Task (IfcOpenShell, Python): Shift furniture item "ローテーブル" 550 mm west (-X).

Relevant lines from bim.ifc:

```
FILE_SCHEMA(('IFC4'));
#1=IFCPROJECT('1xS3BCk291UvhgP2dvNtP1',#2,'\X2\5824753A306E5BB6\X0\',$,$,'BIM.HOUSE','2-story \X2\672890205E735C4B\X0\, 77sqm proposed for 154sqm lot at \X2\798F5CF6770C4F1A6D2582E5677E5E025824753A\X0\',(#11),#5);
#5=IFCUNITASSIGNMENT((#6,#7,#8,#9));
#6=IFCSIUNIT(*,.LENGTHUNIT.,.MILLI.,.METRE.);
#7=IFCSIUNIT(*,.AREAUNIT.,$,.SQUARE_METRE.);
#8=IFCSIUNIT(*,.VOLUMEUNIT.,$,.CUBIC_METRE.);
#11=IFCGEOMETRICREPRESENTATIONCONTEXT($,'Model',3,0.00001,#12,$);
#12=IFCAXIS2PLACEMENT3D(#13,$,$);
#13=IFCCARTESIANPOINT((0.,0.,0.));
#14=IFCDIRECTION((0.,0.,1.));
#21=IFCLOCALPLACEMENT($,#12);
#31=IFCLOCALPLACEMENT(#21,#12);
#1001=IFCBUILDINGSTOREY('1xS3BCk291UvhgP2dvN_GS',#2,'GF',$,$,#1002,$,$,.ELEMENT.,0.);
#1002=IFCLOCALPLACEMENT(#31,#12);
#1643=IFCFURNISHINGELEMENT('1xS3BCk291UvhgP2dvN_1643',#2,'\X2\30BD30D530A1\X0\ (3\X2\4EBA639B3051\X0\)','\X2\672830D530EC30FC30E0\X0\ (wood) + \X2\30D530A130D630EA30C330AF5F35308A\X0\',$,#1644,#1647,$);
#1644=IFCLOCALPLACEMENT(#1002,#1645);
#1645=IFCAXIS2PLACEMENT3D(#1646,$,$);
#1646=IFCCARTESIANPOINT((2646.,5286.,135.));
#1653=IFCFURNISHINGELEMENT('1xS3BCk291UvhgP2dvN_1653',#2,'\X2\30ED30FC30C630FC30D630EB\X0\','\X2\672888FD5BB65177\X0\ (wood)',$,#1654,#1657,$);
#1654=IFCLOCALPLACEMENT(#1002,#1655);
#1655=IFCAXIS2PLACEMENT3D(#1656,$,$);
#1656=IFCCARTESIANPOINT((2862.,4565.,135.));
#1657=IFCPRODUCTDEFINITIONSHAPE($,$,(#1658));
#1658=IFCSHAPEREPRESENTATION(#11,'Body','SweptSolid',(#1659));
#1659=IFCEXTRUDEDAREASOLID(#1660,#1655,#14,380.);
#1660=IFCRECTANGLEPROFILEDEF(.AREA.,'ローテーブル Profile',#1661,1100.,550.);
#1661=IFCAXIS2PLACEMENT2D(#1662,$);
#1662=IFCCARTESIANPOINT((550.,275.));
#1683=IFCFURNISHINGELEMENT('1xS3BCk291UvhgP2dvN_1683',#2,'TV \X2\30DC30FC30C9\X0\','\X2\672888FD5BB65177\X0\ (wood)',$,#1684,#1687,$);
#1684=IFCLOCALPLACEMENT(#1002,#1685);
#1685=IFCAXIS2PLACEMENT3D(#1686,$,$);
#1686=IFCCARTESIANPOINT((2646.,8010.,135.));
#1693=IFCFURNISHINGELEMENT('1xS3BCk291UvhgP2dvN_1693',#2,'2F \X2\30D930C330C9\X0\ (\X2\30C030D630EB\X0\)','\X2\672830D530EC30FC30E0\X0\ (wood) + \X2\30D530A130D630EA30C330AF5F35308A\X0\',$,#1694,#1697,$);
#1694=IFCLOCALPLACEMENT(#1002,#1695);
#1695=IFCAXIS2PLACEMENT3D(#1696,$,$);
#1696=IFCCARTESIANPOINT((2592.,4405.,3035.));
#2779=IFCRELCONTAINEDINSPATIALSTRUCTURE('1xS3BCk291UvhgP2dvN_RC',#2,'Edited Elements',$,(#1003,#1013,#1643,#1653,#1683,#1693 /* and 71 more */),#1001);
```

```python
import ifcopenshell
import ifcopenshell.api.geometry
import ifcopenshell.util.placement

model = ifcopenshell.open("bim.ifc")

item = model.by_guid("1xS3BCk291UvhgP2dvN_1653")
matrix = ifcopenshell.util.placement.get_local_placement(item.ObjectPlacement)
matrix[0, 3] -= 550.0
ifcopenshell.api.geometry.edit_object_placement(model, product=item, matrix=matrix, is_si=False)

print(ifcopenshell.util.placement.get_local_placement(item.ObjectPlacement).round(3) + 0.0)

model.write("bim_updated.ifc")
```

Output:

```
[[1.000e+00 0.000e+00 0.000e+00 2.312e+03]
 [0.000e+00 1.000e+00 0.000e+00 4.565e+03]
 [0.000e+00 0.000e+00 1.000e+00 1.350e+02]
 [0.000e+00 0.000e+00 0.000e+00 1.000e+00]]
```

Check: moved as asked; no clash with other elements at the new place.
